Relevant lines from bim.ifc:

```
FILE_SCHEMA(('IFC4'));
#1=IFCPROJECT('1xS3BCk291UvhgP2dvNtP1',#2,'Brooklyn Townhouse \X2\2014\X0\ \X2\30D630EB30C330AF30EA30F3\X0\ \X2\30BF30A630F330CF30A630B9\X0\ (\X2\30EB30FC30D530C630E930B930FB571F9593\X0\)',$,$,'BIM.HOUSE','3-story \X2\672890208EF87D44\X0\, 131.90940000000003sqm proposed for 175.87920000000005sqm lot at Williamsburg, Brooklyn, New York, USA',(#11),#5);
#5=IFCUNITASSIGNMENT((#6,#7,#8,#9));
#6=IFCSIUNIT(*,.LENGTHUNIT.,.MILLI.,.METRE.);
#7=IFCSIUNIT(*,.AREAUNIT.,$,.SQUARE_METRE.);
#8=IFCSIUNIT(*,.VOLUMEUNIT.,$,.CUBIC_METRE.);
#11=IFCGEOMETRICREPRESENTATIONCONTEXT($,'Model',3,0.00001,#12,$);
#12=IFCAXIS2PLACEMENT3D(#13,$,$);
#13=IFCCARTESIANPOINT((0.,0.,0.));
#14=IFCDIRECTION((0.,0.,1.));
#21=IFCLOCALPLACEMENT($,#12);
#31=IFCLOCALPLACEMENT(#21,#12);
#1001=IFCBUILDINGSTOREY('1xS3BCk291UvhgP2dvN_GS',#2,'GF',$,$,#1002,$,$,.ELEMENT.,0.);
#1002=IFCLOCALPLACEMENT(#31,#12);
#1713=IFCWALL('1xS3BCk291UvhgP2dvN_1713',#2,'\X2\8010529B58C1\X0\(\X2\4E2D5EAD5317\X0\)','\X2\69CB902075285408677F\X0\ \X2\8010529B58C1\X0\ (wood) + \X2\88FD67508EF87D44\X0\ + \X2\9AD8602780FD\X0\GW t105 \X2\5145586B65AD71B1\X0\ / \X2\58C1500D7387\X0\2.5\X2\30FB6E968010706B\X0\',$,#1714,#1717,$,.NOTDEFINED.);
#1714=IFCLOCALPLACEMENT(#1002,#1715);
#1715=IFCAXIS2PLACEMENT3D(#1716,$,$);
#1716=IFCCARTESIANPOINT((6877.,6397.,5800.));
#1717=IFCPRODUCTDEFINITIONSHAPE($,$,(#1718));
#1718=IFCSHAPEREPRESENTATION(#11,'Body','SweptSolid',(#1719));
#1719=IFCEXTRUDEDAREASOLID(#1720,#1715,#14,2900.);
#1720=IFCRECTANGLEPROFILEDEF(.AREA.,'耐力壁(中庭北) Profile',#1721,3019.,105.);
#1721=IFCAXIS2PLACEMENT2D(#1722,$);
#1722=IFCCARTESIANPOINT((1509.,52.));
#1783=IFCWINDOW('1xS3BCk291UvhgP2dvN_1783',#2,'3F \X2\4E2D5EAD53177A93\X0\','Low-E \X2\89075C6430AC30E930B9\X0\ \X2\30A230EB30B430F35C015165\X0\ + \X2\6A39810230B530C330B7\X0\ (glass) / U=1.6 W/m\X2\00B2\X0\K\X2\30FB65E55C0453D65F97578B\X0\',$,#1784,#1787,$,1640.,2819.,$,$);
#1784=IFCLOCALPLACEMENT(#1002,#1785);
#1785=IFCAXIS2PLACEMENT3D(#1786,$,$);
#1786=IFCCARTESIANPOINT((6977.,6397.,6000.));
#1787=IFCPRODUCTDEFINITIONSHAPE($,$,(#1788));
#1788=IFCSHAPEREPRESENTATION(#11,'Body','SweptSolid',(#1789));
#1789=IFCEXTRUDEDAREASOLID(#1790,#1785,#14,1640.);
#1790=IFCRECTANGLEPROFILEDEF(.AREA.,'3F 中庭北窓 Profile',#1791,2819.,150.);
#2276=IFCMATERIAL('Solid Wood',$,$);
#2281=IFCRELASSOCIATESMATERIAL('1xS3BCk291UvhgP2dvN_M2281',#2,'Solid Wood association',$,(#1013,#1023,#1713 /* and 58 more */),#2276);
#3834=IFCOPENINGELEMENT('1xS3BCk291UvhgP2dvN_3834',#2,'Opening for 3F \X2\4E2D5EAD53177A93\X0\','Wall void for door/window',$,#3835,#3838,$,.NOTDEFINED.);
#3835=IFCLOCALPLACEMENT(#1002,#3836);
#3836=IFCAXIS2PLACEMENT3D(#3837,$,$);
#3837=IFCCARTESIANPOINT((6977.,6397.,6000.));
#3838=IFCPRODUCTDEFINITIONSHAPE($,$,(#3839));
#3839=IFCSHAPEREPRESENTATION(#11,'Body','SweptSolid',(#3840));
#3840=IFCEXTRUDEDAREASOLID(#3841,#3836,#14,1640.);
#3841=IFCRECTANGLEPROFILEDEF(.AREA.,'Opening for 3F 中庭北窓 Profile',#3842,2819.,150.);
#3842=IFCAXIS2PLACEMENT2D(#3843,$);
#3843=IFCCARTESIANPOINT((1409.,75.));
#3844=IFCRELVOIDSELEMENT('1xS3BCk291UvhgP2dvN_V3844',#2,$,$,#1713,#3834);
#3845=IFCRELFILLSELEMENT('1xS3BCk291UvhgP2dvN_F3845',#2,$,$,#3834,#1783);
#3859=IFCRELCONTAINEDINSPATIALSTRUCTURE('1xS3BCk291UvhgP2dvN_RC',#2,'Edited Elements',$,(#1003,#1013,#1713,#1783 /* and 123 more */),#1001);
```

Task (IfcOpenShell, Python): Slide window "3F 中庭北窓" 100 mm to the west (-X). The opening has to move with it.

```python
import ifcopenshell
import ifcopenshell.api.geometry
import ifcopenshell.util.placement

model = ifcopenshell.open("bim.ifc")

window = model.by_guid("1xS3BCk291UvhgP2dvN_1783")
opening = window.FillsVoids[0].RelatingOpeningElement
wall = opening.VoidsElements[0].RelatingBuildingElement

wall_matrix = ifcopenshell.util.placement.get_local_placement(wall.ObjectPlacement)
shift = wall_matrix[:3, 0] * -100.0
before = ifcopenshell.util.placement.get_local_placement(window.ObjectPlacement)[:3, 3].copy()

# The window is not placed relative to its opening, so move both.
for product in (opening, window):
    matrix = ifcopenshell.util.placement.get_local_placement(product.ObjectPlacement)
    matrix[:3, 3] += shift
    ifcopenshell.api.geometry.edit_object_placement(model, product=product, matrix=matrix, is_si=False)

after = ifcopenshell.util.placement.get_local_placement(window.ObjectPlacement)[:3, 3]
print("window moved by", (after - before).round(3) + 0.0)

model.write("bim_updated.ifc")
```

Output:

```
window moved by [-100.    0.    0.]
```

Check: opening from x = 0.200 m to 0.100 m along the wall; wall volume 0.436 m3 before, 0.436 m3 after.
